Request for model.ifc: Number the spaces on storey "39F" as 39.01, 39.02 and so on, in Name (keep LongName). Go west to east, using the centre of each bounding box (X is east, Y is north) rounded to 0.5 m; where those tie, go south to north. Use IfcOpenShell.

First a look at what the model holds.

```python
import ifcopenshell
import ifcopenshell.util.element
import ifcopenshell.util.placement

model = ifcopenshell.open("model.ifc")
print(model.schema)
storey = next(s for s in model.by_type("IfcBuildingStorey") if s.Name == "39F")
spaces = [e for e in ifcopenshell.util.element.get_decomposition(storey) if e.is_a("IfcSpace")]
for e in sorted(spaces, key=lambda e: e.id()):
    origin = ifcopenshell.util.placement.get_local_placement(e.ObjectPlacement)[:3, 3]
    print(e.id(), e.Name, e.LongName, origin.round(2) + 0.0, sep=" | ")
```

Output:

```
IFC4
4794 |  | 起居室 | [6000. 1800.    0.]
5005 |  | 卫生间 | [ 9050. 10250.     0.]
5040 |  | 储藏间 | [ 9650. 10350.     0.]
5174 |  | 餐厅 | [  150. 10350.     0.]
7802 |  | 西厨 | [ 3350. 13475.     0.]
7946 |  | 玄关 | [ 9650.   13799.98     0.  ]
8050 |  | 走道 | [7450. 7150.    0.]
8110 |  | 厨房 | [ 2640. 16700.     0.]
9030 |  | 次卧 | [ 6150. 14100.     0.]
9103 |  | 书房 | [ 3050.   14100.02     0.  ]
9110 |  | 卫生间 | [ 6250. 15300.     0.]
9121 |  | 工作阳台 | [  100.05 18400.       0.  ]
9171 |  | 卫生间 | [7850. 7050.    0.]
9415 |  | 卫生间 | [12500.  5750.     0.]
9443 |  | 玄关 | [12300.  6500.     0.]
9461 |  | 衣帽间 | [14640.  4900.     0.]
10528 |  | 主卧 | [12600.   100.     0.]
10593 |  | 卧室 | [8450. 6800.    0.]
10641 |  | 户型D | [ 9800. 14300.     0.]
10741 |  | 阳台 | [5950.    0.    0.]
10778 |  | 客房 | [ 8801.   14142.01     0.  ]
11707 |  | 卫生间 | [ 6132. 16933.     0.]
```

```python
import ifcopenshell
import ifcopenshell.geom
import ifcopenshell.util.element
import ifcopenshell.util.shape

model = ifcopenshell.open("model.ifc")
settings = ifcopenshell.geom.settings()
settings.set("use-world-coords", True)


def centre(element):
    shape = ifcopenshell.geom.create_shape(settings, element)
    return ifcopenshell.util.shape.get_bbox_centroid(shape.geometry)


storey = next(s for s in model.by_type("IfcBuildingStorey") if s.Name == "39F")
spaces = [e for e in ifcopenshell.util.element.get_decomposition(storey) if e.is_a("IfcSpace")]

# Insertion points can sit at a corner or the storey origin, so sort by the geometry (in metres).
centres = {e: centre(e) for e in spaces}
spaces.sort(key=lambda e: (round(centres[e][0] / 0.5), centres[e][1]))

for i, e in enumerate(spaces, start=1):
    number = f"39.{i:02d}"
    e.Name = number
    print(e.id(), number)

model.write("model-out.ifc")
```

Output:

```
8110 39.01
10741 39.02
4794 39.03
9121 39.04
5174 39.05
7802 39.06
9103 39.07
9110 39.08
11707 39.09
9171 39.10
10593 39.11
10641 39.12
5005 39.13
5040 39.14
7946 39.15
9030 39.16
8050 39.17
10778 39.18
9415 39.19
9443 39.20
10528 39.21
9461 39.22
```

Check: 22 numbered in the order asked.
